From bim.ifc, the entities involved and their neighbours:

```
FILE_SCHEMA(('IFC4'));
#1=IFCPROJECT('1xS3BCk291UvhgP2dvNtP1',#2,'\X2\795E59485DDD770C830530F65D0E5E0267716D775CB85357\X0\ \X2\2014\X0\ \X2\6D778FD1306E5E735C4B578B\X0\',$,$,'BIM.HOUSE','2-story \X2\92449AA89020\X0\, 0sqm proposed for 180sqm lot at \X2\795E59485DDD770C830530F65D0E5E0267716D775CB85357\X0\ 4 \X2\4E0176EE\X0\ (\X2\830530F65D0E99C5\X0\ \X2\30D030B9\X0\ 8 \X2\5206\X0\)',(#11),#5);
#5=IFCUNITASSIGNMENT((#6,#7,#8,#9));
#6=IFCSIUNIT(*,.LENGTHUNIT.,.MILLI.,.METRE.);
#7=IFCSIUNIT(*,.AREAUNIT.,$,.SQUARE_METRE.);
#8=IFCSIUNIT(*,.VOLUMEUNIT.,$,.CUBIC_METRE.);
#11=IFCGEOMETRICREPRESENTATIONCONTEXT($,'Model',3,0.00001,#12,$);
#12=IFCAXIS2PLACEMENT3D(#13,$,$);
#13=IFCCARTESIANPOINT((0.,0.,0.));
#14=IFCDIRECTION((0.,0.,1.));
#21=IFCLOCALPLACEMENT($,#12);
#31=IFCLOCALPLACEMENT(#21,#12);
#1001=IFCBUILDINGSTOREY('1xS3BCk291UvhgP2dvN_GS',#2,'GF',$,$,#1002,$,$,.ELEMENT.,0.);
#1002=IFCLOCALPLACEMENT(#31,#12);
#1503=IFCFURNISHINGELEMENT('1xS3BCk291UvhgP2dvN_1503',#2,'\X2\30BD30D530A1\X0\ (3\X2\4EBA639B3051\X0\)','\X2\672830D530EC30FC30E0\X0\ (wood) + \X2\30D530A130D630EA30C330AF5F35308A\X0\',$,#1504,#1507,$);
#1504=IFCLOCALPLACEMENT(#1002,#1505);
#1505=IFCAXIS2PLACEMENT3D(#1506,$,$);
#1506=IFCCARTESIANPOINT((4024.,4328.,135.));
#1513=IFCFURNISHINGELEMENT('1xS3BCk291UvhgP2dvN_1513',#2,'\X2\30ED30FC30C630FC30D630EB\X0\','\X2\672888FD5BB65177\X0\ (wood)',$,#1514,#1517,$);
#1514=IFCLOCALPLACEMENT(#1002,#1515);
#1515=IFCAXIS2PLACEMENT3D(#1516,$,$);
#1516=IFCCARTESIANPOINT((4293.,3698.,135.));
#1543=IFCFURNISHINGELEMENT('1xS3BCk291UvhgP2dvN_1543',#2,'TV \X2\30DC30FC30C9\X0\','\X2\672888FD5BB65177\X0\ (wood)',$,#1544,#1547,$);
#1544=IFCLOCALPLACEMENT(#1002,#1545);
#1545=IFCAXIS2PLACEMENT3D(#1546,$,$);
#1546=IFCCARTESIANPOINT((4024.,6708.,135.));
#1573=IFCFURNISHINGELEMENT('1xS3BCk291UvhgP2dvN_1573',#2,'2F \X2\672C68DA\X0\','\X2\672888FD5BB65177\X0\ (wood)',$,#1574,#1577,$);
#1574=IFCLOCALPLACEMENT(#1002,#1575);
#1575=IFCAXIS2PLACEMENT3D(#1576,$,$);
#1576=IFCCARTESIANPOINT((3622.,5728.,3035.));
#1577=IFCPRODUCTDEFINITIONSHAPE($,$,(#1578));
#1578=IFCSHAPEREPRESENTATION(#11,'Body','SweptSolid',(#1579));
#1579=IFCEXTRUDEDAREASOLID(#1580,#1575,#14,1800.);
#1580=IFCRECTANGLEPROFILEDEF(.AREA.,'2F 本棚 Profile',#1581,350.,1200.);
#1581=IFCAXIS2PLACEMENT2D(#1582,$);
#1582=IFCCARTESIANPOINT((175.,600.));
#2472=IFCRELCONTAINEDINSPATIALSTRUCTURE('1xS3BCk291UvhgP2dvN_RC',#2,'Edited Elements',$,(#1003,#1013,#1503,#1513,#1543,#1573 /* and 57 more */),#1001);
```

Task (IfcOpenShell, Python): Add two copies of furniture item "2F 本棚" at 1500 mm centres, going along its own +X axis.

```python
import ifcopenshell
import ifcopenshell.api.geometry
import ifcopenshell.api.root
import ifcopenshell.util.element
import ifcopenshell.util.placement
import ifcopenshell.util.unit

model = ifcopenshell.open("bim.ifc")
unit_scale = ifcopenshell.util.unit.calculate_unit_scale(model)


def reuse_history(source, copy):
    """copy_class also copies each property set's owner history, people and application; keep the originals."""
    for rel in copy.IsDefinedBy:
        if rel.is_a("IfcRelDefinesByProperties") and (history := rel.RelatingPropertyDefinition.OwnerHistory):
            rel.RelatingPropertyDefinition.OwnerHistory = source.OwnerHistory
            ifcopenshell.util.element.remove_deep2(model, history)


source = model.by_guid("1xS3BCk291UvhgP2dvN_1573")
base = ifcopenshell.util.placement.get_local_placement(source.ObjectPlacement)
step = base[:3, 0] * 1.5 / unit_scale

for i in range(1, 3):
    copy = ifcopenshell.api.root.copy_class(model, product=source)
    copy.Representation = ifcopenshell.util.element.copy_deep(
        model, source.Representation, exclude=["IfcGeometricRepresentationContext", "IfcRepresentationMap"]
    )
    reuse_history(source, copy)
    matrix = base.copy()
    matrix[:3, 3] += i * step
    print("added at", matrix[:3, 3].round(3) + 0.0)
    ifcopenshell.api.geometry.edit_object_placement(model, product=copy, matrix=matrix, is_si=False)

model.write("bim_v2.ifc")
```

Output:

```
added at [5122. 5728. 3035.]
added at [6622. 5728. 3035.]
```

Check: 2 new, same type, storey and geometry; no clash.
